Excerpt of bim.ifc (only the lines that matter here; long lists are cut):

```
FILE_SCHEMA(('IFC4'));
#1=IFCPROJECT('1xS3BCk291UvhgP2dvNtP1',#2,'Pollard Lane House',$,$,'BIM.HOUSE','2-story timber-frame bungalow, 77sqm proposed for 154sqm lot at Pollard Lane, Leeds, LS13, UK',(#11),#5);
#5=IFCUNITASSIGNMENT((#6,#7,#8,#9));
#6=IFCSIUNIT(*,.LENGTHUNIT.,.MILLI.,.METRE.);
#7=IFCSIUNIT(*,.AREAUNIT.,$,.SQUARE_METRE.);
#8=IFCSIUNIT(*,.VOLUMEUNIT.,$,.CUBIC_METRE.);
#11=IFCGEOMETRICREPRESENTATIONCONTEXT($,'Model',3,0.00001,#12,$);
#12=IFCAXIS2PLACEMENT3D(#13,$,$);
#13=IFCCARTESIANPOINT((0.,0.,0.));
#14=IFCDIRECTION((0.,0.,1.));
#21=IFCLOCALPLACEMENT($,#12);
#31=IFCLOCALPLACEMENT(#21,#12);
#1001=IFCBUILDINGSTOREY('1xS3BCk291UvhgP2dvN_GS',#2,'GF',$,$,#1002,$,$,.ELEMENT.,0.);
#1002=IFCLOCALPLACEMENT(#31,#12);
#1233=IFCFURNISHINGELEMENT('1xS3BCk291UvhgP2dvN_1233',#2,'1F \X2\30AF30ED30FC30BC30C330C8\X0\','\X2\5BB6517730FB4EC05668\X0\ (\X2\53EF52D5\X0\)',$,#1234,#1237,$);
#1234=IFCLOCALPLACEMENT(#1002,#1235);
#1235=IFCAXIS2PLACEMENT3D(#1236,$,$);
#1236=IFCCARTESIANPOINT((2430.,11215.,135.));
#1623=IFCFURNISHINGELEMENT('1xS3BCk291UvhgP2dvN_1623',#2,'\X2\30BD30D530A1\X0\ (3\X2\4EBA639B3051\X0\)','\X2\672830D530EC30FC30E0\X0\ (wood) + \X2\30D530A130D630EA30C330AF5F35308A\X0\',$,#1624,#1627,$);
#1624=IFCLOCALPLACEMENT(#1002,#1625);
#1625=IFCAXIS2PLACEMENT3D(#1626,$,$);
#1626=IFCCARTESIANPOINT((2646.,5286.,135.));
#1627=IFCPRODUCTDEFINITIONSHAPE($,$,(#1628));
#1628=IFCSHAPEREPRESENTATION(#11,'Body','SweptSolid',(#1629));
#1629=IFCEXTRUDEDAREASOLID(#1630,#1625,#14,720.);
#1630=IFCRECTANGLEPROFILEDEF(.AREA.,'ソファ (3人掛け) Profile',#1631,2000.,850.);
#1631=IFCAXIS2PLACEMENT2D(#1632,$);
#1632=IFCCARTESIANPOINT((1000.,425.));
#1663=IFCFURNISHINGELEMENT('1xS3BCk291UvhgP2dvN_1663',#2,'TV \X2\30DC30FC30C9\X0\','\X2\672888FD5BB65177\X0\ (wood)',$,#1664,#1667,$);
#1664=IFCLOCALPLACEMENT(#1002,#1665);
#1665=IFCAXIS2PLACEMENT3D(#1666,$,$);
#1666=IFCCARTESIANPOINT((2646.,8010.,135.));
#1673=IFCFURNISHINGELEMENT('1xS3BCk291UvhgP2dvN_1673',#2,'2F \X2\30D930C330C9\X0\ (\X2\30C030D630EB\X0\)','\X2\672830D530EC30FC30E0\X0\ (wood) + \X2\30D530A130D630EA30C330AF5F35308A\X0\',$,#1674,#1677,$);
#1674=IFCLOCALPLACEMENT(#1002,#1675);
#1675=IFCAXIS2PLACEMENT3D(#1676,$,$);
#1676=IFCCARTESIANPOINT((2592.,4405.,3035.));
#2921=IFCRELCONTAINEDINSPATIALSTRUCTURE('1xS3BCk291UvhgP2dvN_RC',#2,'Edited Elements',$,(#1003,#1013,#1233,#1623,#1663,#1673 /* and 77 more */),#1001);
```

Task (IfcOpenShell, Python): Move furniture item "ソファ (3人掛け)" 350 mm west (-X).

```python
import ifcopenshell
import ifcopenshell.api.geometry
import ifcopenshell.util.placement
import ifcopenshell.util.unit

model = ifcopenshell.open("bim.ifc")
unit_scale = ifcopenshell.util.unit.calculate_unit_scale(model)

item = model.by_guid("1xS3BCk291UvhgP2dvN_1623")
matrix = ifcopenshell.util.placement.get_local_placement(item.ObjectPlacement)
matrix[0, 3] -= 0.35 / unit_scale
ifcopenshell.api.geometry.edit_object_placement(model, product=item, matrix=matrix, is_si=False)

print(ifcopenshell.util.placement.get_local_placement(item.ObjectPlacement).round(3) + 0.0)

model.write("bim_rev.ifc")
```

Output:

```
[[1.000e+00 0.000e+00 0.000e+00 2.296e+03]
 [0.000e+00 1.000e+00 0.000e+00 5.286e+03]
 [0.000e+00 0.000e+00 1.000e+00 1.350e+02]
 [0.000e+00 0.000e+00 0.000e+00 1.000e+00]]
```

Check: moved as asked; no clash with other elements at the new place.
